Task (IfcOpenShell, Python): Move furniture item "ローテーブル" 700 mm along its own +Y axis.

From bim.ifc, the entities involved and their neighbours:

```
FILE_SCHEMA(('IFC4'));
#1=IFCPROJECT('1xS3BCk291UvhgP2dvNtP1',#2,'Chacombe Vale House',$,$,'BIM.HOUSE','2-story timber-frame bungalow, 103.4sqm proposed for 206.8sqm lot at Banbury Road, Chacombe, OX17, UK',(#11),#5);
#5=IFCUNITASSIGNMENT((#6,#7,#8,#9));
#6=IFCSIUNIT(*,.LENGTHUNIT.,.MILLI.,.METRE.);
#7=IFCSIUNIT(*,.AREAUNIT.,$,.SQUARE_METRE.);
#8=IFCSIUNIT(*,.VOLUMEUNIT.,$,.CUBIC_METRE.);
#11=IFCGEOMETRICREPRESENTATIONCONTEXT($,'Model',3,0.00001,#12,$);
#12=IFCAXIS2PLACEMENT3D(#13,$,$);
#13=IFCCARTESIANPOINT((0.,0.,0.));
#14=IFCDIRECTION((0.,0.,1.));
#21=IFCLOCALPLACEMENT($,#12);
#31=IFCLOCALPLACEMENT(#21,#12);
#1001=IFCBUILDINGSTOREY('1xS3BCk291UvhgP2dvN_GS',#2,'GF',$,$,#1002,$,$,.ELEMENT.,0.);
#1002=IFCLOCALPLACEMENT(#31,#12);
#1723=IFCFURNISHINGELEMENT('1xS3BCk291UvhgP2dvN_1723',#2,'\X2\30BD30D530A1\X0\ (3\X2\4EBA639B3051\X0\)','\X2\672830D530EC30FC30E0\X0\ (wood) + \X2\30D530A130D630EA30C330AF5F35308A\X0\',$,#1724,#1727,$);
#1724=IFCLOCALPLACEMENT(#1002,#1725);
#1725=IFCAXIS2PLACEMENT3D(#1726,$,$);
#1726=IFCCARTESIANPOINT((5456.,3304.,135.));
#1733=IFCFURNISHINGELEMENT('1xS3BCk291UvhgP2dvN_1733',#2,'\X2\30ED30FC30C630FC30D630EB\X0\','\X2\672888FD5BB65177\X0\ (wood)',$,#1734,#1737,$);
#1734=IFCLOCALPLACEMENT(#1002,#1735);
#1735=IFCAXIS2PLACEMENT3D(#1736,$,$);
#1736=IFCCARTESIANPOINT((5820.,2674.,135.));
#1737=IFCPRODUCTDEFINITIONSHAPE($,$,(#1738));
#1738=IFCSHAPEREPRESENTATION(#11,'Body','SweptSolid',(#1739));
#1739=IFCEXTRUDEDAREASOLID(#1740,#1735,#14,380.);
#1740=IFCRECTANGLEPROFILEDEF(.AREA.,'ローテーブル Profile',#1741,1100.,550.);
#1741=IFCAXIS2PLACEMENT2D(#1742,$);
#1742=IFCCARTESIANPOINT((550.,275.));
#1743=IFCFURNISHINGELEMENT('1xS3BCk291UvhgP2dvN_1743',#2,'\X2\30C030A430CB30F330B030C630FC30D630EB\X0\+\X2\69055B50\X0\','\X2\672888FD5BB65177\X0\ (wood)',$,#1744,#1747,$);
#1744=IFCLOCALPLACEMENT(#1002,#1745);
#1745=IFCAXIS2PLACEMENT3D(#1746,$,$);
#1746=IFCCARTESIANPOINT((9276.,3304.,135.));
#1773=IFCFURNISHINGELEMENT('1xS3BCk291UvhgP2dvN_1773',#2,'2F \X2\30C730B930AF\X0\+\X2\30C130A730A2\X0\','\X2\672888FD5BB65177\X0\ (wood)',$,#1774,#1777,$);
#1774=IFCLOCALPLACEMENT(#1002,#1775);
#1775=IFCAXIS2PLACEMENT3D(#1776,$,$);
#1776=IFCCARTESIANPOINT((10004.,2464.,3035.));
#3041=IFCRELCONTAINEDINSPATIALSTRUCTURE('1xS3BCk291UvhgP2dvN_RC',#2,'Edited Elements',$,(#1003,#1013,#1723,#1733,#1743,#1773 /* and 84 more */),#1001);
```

```python
import ifcopenshell
import ifcopenshell.api.geometry
import ifcopenshell.util.placement
import ifcopenshell.util.unit

model = ifcopenshell.open("bim.ifc")
unit_scale = ifcopenshell.util.unit.calculate_unit_scale(model)

item = model.by_guid("1xS3BCk291UvhgP2dvN_1733")
matrix = ifcopenshell.util.placement.get_local_placement(item.ObjectPlacement)
matrix[:3, 3] += matrix[:3, 1] * 0.7 / unit_scale
ifcopenshell.api.geometry.edit_object_placement(model, product=item, matrix=matrix, is_si=False)

print(ifcopenshell.util.placement.get_local_placement(item.ObjectPlacement).round(3) + 0.0)

model.write("bim_updated.ifc")
```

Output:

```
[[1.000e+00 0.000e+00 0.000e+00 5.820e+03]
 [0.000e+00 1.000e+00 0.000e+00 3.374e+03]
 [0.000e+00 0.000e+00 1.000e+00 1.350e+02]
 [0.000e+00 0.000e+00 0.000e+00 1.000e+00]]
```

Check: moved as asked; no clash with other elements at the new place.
